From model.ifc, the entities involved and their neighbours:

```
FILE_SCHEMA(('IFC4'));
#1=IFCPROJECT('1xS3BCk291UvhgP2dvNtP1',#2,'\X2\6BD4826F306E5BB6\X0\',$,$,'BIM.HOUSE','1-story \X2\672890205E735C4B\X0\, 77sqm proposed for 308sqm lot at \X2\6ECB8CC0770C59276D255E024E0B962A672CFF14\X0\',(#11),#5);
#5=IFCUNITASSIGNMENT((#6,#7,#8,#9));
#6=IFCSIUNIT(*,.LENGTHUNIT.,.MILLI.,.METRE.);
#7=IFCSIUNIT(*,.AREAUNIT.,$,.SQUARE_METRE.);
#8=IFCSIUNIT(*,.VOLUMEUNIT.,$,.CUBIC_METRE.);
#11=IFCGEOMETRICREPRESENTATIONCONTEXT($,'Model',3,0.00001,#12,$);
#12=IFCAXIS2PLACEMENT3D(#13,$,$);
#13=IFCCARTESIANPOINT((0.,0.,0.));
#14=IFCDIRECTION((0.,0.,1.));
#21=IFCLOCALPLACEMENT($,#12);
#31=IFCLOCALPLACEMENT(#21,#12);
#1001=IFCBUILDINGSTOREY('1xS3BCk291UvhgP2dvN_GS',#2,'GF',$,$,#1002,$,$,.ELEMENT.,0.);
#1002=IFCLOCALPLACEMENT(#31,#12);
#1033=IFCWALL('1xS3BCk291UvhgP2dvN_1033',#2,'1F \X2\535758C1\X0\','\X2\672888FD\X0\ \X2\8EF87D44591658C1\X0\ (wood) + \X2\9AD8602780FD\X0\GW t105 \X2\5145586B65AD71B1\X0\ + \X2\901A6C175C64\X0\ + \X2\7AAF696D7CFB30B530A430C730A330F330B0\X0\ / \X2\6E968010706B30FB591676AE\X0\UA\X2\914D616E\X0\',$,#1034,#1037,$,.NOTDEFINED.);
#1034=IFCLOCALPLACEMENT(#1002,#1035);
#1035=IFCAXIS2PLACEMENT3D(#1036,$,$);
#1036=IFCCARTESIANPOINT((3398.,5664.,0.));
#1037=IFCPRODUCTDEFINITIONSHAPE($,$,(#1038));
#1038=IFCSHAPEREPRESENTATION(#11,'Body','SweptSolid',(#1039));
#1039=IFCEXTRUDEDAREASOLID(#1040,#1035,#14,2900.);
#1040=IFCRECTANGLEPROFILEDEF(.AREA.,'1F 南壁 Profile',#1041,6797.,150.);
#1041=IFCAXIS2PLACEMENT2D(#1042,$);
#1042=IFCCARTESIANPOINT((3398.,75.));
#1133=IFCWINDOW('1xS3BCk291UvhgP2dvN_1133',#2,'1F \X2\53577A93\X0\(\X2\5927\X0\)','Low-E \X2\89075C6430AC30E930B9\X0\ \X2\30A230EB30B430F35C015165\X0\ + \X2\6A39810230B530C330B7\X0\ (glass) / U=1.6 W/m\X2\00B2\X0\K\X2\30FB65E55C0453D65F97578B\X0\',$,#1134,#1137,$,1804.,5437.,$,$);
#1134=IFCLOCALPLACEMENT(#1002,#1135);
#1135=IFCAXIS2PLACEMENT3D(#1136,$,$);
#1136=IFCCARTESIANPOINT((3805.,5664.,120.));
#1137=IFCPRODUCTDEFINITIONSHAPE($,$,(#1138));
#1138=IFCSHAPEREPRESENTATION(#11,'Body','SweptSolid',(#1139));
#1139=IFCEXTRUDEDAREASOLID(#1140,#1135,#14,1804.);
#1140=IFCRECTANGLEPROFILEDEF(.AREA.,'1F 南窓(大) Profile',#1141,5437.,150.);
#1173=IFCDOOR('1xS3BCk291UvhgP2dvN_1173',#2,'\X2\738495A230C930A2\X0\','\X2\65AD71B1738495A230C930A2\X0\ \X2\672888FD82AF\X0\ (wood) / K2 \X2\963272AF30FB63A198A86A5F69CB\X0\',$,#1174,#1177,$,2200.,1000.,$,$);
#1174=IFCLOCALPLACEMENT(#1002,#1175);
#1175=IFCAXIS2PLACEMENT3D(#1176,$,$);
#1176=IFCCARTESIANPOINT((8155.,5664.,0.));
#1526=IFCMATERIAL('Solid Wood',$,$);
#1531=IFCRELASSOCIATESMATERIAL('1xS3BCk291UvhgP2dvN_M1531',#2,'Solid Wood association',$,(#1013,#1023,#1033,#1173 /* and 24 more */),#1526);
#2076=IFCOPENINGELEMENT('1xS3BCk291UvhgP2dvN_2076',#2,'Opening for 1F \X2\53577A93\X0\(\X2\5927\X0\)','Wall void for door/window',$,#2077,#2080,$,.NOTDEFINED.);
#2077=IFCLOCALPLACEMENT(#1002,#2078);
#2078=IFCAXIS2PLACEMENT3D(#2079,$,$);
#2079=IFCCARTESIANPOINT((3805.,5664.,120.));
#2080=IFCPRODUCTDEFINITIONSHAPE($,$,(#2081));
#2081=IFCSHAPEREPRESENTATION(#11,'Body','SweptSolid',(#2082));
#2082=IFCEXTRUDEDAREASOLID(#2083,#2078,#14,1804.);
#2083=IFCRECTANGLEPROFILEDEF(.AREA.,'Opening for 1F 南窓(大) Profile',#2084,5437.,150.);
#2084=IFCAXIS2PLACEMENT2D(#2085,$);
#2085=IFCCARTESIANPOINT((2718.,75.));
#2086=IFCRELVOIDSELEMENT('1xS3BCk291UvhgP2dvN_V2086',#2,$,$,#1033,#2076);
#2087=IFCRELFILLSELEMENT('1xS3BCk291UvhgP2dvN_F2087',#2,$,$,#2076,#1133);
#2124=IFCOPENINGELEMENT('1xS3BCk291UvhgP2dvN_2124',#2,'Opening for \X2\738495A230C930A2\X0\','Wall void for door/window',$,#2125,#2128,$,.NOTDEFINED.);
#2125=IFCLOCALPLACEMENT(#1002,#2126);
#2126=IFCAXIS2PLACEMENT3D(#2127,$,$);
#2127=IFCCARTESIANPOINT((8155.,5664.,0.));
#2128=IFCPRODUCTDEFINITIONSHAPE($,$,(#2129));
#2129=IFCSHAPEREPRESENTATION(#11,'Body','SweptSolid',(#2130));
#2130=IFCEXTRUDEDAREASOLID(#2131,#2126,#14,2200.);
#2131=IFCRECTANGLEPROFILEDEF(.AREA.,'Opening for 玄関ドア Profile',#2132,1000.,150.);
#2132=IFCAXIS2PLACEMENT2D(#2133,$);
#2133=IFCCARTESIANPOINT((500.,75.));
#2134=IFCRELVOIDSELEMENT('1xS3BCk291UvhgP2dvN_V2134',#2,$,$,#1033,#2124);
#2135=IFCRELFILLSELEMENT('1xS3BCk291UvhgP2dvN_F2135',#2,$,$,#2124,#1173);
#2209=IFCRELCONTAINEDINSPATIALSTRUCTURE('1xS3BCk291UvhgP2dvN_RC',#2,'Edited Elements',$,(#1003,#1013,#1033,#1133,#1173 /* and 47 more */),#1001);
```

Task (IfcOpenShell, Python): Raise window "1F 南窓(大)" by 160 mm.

```python
import numpy as np
import ifcopenshell
import ifcopenshell.api.geometry
import ifcopenshell.util.placement
import ifcopenshell.util.unit

model = ifcopenshell.open("model.ifc")
unit_scale = ifcopenshell.util.unit.calculate_unit_scale(model)

window = model.by_id(1133)
opening = window.FillsVoids[0].RelatingOpeningElement
dz = 160.0

shift = np.array([0.0, 0.0, dz])
# The window is not placed relative to its opening, so move both.
for product in (opening, window):
    matrix = ifcopenshell.util.placement.get_local_placement(product.ObjectPlacement)
    matrix[:3, 3] += shift
    ifcopenshell.api.geometry.edit_object_placement(model, product=product, matrix=matrix, is_si=False)

print(f"moved by {dz * unit_scale:+.3f} m")

model.write("model_edited.ifc")
```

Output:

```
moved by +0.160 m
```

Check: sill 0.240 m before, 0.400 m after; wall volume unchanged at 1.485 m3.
